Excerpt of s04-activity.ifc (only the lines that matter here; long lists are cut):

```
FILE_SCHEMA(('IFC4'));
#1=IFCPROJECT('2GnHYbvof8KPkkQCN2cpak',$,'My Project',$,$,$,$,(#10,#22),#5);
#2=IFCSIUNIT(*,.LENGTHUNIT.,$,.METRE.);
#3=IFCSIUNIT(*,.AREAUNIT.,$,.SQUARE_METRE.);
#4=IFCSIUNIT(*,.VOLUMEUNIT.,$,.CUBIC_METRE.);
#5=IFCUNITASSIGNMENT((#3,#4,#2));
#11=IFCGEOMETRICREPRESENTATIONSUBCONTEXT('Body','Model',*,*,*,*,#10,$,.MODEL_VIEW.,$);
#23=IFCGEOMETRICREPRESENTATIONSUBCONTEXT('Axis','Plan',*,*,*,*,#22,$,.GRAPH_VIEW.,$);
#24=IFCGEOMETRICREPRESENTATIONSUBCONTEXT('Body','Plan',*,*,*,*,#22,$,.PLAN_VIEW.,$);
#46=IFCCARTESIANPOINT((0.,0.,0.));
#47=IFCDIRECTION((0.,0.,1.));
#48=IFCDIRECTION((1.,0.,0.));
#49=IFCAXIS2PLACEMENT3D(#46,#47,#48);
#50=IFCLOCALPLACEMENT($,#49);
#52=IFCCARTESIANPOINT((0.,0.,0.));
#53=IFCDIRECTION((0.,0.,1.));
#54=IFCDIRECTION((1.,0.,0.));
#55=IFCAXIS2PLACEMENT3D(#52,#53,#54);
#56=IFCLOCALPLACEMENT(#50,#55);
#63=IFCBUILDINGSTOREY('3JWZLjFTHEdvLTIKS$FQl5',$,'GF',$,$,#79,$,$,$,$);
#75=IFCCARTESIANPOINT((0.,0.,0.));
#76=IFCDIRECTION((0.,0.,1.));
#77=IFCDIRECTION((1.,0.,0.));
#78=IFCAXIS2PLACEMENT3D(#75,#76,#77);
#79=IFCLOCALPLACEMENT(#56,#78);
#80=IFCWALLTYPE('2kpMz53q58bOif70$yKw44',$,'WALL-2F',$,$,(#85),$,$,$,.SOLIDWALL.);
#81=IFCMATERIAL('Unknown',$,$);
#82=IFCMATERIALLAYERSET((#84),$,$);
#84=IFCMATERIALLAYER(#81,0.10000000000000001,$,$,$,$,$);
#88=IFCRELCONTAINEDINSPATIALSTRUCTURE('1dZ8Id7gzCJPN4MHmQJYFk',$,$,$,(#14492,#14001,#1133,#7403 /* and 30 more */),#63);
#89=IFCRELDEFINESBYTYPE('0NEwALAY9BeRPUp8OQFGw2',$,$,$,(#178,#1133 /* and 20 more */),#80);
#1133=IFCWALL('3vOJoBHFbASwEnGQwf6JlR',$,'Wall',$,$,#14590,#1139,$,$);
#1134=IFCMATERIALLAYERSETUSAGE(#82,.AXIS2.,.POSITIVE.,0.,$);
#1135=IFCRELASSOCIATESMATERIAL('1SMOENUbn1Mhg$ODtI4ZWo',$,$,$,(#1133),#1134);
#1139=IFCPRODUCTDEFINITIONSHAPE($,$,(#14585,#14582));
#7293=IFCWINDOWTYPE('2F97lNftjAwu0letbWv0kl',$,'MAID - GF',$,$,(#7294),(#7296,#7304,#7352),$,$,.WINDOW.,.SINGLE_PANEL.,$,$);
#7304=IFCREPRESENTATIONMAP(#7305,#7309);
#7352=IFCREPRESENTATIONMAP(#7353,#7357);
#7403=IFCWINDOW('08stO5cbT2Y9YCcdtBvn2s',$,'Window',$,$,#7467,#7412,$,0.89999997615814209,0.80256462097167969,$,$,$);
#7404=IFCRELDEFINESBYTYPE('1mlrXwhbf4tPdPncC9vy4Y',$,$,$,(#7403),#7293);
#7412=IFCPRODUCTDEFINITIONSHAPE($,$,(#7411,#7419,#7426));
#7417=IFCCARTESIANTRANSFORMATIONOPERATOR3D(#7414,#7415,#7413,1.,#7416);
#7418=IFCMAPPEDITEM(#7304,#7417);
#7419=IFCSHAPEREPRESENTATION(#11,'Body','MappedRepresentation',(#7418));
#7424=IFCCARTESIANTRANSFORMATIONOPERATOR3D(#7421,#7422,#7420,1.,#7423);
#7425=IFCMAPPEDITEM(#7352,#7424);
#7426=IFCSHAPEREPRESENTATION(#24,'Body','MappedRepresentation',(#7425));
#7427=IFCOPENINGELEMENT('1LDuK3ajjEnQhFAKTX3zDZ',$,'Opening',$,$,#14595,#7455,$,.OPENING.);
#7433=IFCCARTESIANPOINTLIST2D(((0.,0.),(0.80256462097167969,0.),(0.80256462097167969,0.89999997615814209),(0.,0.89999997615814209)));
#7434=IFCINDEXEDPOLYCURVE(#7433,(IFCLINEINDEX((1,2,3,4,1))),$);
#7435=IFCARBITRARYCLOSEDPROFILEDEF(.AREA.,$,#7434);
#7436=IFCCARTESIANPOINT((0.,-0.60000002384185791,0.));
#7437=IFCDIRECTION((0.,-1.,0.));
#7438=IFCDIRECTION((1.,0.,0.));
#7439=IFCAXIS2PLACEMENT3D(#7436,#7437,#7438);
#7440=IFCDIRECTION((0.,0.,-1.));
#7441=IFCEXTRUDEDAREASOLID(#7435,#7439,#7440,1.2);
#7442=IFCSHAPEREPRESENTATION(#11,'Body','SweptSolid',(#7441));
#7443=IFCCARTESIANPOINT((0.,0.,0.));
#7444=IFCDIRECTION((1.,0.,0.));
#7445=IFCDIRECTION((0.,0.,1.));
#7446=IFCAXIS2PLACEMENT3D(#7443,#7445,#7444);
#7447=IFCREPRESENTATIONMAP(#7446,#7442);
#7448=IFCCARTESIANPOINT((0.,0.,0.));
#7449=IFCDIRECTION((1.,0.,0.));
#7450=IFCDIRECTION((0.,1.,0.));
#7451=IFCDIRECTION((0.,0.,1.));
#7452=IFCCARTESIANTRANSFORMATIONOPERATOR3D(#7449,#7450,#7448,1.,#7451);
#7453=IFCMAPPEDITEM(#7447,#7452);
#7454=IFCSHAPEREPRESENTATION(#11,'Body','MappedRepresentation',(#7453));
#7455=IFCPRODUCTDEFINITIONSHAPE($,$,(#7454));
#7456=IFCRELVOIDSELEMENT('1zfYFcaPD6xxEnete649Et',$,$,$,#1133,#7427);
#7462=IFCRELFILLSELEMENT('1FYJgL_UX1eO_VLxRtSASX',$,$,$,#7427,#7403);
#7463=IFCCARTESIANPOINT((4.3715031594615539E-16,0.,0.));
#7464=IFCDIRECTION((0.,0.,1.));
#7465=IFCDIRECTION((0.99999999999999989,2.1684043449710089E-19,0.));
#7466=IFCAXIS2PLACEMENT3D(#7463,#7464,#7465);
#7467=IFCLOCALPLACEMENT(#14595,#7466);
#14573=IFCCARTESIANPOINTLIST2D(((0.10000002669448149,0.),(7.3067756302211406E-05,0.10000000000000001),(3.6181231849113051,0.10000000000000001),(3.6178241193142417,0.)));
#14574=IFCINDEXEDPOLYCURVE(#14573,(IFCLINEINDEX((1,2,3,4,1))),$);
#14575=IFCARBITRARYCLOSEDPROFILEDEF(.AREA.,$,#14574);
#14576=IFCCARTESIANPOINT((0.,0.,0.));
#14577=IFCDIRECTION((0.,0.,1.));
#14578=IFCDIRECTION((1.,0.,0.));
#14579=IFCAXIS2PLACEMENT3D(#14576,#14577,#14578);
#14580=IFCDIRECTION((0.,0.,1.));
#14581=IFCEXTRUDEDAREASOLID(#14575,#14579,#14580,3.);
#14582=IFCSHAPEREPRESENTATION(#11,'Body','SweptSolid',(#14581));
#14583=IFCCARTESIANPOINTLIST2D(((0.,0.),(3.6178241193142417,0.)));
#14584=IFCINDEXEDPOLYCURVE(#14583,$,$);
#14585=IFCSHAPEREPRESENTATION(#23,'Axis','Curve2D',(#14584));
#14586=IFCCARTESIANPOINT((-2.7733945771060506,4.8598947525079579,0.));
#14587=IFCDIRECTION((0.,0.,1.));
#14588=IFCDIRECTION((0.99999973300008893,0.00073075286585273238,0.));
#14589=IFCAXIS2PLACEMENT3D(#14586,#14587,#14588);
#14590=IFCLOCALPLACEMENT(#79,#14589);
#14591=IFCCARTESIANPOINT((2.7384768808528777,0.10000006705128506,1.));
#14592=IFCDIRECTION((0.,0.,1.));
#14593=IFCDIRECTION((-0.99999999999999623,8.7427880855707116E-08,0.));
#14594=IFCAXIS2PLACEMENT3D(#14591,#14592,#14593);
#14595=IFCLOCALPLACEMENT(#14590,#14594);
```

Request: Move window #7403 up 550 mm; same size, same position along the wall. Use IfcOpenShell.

```python
import numpy as np
import ifcopenshell
import ifcopenshell.api.geometry
import ifcopenshell.util.placement
import ifcopenshell.util.unit

model = ifcopenshell.open("s04-activity.ifc")
unit_scale = ifcopenshell.util.unit.calculate_unit_scale(model)

window = model.by_guid("08stO5cbT2Y9YCcdtBvn2s")
opening = window.FillsVoids[0].RelatingOpeningElement
dz = 0.55 / unit_scale

shift = np.array([0.0, 0.0, dz])
# The window is placed relative to its opening, so it follows when the opening moves.
matrix = ifcopenshell.util.placement.get_local_placement(opening.ObjectPlacement)
matrix[:3, 3] += shift
ifcopenshell.api.geometry.edit_object_placement(
    model, product=opening, matrix=matrix, is_si=False, should_transform_children=True
)

print(f"moved by {dz * unit_scale:+.3f} m")

model.write("s04-activity-out.ifc")
```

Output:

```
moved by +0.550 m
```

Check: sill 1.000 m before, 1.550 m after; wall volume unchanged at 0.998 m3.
